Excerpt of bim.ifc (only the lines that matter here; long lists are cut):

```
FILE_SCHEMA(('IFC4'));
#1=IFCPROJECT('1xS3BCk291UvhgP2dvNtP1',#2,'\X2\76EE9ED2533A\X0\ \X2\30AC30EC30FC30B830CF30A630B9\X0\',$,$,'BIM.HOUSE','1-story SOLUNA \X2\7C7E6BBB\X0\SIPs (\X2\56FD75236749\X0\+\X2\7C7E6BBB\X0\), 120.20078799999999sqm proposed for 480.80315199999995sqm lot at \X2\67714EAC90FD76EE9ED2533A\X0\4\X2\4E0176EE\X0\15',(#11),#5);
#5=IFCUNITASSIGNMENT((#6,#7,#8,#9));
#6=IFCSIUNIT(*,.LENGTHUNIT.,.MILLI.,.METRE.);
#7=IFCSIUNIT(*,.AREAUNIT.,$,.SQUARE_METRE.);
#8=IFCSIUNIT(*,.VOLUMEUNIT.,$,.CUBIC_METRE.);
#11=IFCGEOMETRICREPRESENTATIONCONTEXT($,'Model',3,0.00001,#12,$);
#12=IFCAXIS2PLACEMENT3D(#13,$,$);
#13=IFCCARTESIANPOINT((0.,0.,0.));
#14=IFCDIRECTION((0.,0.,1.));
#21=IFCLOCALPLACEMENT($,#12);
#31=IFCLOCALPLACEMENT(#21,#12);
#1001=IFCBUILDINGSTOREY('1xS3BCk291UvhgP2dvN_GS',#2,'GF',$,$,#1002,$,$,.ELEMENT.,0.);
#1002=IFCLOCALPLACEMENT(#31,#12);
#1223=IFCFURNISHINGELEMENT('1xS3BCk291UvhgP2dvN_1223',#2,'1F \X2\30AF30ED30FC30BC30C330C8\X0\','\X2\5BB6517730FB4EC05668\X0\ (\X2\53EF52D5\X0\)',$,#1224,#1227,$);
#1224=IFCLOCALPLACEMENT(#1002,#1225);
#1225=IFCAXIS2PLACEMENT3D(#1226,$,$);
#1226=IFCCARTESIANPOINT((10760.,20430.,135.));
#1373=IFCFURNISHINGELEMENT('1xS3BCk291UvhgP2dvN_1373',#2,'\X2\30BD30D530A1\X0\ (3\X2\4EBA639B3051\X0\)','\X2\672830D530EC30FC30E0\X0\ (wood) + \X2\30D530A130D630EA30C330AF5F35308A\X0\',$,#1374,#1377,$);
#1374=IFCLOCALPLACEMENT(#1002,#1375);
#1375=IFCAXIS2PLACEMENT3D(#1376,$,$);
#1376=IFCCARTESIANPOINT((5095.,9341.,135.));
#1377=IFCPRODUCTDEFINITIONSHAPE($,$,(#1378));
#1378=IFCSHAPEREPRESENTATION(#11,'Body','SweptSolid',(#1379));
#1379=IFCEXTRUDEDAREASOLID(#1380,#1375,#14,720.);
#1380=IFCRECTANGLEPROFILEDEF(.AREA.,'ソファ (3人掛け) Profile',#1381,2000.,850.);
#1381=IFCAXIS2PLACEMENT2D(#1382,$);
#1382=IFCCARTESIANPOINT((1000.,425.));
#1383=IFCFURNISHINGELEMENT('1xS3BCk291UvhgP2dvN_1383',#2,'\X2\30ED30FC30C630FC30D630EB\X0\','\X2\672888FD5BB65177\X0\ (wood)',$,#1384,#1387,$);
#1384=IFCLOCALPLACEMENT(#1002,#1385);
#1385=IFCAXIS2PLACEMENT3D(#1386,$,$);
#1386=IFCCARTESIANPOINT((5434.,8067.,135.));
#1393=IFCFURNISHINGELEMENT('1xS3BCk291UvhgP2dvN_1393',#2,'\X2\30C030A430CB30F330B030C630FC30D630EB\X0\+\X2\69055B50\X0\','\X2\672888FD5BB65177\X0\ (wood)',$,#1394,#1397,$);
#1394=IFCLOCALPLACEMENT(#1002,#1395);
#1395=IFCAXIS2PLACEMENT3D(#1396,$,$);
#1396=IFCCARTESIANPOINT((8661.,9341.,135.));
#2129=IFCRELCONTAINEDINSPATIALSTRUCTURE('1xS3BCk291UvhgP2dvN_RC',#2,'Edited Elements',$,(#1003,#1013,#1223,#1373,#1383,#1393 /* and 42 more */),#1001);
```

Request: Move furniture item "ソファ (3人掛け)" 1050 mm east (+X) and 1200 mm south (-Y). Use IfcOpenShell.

```python
import ifcopenshell
import ifcopenshell.api.geometry
import ifcopenshell.util.placement
import ifcopenshell.util.unit

model = ifcopenshell.open("bim.ifc")
unit_scale = ifcopenshell.util.unit.calculate_unit_scale(model)

item = model.by_guid("1xS3BCk291UvhgP2dvN_1373")
matrix = ifcopenshell.util.placement.get_local_placement(item.ObjectPlacement)
matrix[0, 3] += 1.05 / unit_scale
matrix[1, 3] -= 1.2 / unit_scale
ifcopenshell.api.geometry.edit_object_placement(model, product=item, matrix=matrix, is_si=False)

print(ifcopenshell.util.placement.get_local_placement(item.ObjectPlacement).round(3) + 0.0)

model.write("bim_edited.ifc")
```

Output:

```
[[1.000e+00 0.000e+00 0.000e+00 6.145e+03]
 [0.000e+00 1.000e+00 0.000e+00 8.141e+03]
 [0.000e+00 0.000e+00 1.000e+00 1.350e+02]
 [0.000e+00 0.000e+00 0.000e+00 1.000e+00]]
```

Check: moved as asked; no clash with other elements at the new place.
